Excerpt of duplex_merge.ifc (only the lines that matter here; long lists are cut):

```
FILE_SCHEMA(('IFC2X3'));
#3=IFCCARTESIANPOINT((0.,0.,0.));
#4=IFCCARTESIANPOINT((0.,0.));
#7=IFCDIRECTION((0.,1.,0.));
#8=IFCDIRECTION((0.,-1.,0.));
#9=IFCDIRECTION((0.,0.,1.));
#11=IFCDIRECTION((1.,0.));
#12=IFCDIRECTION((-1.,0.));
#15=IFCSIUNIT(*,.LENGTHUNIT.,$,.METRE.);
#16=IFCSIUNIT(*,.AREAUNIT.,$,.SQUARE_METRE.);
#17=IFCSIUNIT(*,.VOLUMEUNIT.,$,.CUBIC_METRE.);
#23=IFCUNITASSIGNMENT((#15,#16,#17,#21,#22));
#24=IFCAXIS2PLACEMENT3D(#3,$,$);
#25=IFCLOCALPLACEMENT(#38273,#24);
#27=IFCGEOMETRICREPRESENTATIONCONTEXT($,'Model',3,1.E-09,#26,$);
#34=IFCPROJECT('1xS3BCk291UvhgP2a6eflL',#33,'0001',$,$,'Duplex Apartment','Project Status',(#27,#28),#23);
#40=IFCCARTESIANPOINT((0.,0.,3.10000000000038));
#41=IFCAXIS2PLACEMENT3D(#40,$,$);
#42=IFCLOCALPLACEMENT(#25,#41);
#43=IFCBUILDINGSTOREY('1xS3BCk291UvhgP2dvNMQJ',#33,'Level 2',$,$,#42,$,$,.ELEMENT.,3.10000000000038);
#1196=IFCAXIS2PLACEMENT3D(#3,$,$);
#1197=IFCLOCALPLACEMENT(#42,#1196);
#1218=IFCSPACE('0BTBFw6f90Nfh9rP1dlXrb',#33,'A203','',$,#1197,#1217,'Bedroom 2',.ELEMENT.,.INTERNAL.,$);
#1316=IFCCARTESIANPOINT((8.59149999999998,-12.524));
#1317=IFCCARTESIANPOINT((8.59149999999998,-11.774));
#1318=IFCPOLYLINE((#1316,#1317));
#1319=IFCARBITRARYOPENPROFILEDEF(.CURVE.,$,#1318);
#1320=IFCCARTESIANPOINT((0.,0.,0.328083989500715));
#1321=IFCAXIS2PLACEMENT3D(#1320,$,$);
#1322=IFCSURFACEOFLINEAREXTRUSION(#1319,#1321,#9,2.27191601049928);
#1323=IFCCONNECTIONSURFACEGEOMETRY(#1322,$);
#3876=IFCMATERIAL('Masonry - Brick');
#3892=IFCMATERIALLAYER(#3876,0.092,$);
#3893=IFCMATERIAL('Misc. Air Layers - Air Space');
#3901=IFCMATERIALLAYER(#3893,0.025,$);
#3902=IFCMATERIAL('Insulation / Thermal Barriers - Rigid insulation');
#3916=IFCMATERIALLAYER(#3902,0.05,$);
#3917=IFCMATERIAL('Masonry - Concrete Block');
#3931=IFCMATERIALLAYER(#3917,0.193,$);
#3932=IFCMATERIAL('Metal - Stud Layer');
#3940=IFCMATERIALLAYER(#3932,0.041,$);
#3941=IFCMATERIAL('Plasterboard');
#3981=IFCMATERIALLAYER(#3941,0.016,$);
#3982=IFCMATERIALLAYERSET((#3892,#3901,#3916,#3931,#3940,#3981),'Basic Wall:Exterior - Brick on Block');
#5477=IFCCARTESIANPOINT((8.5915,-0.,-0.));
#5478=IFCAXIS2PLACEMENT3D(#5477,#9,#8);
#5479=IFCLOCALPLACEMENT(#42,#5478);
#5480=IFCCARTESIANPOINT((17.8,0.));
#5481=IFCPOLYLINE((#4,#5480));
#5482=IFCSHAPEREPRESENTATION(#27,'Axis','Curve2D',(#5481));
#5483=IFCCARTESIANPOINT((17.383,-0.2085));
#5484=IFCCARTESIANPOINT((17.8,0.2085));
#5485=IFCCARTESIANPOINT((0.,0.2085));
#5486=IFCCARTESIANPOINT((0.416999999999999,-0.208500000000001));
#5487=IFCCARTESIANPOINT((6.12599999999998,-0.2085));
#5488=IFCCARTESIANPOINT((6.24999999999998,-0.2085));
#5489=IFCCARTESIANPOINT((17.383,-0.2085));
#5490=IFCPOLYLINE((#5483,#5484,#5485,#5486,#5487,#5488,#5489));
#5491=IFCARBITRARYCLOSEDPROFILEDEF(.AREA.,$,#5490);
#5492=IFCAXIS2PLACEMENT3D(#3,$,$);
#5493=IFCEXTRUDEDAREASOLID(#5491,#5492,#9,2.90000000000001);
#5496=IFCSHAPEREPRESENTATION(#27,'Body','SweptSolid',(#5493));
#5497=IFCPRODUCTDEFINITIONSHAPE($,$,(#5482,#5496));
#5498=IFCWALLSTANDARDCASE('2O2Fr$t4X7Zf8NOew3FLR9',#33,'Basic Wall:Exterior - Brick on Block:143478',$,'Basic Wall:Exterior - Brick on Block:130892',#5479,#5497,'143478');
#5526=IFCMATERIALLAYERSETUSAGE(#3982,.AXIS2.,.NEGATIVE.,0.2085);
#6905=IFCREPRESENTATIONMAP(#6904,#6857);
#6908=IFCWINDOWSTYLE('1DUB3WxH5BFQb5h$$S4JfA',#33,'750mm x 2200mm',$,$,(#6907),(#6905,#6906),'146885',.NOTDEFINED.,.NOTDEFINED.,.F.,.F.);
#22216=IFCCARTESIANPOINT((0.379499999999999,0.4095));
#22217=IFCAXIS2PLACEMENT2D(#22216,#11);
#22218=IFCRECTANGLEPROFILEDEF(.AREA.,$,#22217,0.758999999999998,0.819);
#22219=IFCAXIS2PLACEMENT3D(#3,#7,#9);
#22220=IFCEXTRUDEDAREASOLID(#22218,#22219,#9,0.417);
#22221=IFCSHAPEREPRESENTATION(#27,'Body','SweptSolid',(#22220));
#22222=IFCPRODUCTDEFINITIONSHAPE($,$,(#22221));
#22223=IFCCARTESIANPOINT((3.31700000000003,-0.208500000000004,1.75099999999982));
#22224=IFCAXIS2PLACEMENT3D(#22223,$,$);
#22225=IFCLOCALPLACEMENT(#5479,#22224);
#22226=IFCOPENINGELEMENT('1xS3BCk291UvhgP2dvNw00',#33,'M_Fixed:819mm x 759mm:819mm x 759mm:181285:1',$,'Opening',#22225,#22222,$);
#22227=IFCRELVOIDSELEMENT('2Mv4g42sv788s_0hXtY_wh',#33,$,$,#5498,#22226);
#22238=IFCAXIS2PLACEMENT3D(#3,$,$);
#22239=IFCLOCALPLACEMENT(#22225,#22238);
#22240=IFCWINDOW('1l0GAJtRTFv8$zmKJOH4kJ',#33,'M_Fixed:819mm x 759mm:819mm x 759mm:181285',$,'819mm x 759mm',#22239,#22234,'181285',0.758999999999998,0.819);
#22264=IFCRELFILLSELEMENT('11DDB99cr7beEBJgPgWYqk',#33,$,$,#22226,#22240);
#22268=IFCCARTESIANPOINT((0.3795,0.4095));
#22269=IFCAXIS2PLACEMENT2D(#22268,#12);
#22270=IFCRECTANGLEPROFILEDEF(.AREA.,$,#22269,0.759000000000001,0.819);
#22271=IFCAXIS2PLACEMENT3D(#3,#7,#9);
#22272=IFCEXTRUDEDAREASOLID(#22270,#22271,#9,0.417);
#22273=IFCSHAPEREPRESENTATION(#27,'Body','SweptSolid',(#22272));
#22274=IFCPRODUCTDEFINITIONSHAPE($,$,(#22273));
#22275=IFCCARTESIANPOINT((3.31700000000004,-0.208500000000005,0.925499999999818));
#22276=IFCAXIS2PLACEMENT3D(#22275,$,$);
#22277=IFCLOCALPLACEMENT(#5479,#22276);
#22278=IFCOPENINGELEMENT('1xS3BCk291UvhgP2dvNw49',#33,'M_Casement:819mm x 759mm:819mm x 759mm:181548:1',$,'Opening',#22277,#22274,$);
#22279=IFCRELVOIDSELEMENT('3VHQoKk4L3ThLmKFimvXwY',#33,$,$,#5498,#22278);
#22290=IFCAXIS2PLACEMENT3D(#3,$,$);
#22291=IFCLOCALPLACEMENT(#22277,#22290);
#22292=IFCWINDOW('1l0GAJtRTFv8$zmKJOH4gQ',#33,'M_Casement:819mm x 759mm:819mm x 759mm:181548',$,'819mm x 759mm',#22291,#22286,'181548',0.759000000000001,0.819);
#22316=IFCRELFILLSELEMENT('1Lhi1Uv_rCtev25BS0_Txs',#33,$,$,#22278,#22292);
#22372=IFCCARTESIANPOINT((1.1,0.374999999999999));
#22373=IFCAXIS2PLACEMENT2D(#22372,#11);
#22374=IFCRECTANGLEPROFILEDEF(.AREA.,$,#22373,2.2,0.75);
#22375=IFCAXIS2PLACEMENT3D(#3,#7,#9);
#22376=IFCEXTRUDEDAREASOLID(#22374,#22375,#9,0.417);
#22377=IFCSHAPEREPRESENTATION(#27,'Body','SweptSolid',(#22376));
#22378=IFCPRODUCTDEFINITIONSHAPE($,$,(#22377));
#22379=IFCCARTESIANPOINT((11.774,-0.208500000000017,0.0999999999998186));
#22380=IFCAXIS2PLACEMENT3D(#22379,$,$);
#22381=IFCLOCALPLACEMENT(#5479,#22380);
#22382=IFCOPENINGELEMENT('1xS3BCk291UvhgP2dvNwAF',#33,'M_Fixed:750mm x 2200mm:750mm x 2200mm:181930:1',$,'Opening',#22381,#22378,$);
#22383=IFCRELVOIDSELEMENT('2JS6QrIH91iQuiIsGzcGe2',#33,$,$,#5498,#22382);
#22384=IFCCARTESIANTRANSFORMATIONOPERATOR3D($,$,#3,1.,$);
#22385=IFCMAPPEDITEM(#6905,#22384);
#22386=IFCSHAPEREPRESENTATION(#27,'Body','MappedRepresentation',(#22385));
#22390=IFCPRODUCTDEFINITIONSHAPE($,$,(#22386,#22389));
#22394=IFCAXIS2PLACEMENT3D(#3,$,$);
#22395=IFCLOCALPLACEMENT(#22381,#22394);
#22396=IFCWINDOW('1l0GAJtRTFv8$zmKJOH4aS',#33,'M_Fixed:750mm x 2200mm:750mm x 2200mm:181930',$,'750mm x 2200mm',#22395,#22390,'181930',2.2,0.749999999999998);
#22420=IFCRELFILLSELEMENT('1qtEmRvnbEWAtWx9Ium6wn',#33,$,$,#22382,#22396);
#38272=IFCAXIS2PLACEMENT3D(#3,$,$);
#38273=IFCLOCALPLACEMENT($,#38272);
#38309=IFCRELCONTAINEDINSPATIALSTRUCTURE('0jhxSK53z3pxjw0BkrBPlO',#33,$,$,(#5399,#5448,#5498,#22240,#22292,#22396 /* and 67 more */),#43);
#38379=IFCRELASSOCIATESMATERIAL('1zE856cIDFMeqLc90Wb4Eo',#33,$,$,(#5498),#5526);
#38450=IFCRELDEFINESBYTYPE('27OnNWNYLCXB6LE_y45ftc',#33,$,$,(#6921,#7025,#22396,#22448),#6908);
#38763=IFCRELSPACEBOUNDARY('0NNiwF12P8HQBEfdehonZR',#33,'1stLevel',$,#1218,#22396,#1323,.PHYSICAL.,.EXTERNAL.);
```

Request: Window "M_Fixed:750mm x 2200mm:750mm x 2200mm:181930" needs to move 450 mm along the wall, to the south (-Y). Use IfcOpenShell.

```python
import numpy as np
import ifcopenshell
import ifcopenshell.api.geometry
import ifcopenshell.util.placement
import ifcopenshell.util.unit

model = ifcopenshell.open("duplex_merge.ifc")
unit_scale = ifcopenshell.util.unit.calculate_unit_scale(model)

window = model.by_guid("1l0GAJtRTFv8$zmKJOH4aS")
opening = window.FillsVoids[0].RelatingOpeningElement
wall = opening.VoidsElements[0].RelatingBuildingElement

wall_matrix = ifcopenshell.util.placement.get_local_placement(wall.ObjectPlacement)
shift = wall_matrix[:3, 0] * 0.45 / unit_scale
before = ifcopenshell.util.placement.get_local_placement(window.ObjectPlacement)[:3, 3].copy()

# The window is placed relative to its opening, so it follows when the opening moves.
matrix = ifcopenshell.util.placement.get_local_placement(opening.ObjectPlacement)
matrix[:3, 3] += shift
ifcopenshell.api.geometry.edit_object_placement(
    model, product=opening, matrix=matrix, is_si=False, should_transform_children=True
)

# Space boundary surfaces are stored in each space's coordinates; move them too.
for rel in window.ProvidesBoundaries:
    if not rel.ConnectionGeometry:
        continue
    surface = rel.ConnectionGeometry.SurfaceOnRelatingElement
    space_matrix = ifcopenshell.util.placement.get_local_placement(rel.RelatingSpace.ObjectPlacement)
    point = np.array(surface.Position.Location.Coordinates) + space_matrix[:3, :3].T @ shift
    surface.Position = model.createIfcAxis2Placement3D(
        model.createIfcCartesianPoint(point.tolist()), surface.Position.Axis, surface.Position.RefDirection
    )

after = ifcopenshell.util.placement.get_local_placement(window.ObjectPlacement)[:3, 3]
print("window moved by", (after - before).round(3) + 0.0)

model.write("duplex_merge_edited.ifc")
```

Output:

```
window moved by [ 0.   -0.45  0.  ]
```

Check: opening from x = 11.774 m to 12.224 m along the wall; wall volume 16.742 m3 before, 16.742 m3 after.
